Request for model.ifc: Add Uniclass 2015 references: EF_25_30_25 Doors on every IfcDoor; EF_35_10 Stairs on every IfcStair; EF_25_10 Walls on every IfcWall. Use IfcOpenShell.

First a look at what the model holds.

```python
import ifcopenshell

model = ifcopenshell.open("model.ifc")
print(model.schema)
print("classifications:", [c.Name for c in model.by_type("IfcClassification")])
for ifc_class in ("IfcDoor", "IfcRoof", "IfcStair", "IfcWall", "IfcWindow"):
    print(ifc_class, len(model.by_type(ifc_class)))
```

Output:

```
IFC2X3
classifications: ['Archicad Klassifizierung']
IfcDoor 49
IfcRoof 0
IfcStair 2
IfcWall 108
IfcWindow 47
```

```python
import ifcopenshell
import ifcopenshell.api.classification

model = ifcopenshell.open("model.ifc")

# IFC2X3 requires Source and Edition and has no link from the project to the system.
system = model.create_entity("IfcClassification", Source="NBS", Edition="2015", Name="Uniclass 2015")

codes = {
    "IfcDoor": ("EF_25_30_25", "Doors"),
    "IfcStair": ("EF_35_10", "Stairs"),
    "IfcWall": ("EF_25_10", "Walls"),
}
for ifc_class, (code, name) in codes.items():
    products = model.by_type(ifc_class)
    ifcopenshell.api.classification.add_reference(
        model, products=products, classification=system, identification=code, name=name
    )
    print(code, len(products))

model.write("model_v2.ifc")
```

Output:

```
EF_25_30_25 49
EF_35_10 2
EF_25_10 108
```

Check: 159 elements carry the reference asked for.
